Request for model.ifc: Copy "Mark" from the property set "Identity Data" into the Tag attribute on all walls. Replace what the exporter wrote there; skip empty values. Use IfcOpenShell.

First a look at what the model holds.

```python
import ifcopenshell
import ifcopenshell.util.element

model = ifcopenshell.open("model.ifc")
print(model.schema)
walls = model.by_type("IfcWall")
print(len(walls), "walls")
for e in walls[:8]:
    source = ifcopenshell.util.element.get_pset(e, "Identity Data", "Mark")
    target = e.Tag
    print(e.id(), repr(source), repr(target), sep=" | ")
```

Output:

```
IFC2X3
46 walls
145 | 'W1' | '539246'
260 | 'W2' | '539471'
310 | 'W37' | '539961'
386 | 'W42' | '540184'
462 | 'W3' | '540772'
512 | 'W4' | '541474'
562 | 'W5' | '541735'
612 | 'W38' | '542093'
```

```python
import ifcopenshell
import ifcopenshell.util.element

model = ifcopenshell.open("model.ifc")

count = 0
for e in model.by_type("IfcWall"):
    value = ifcopenshell.util.element.get_pset(e, "Identity Data", "Mark")
    current = e.Tag
    if not value or not value.strip() or current == value:
        continue
    e.Tag = value
    count += 1

print(count, "walls updated")

model.write("model_rev.ifc")
```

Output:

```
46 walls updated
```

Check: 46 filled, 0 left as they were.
